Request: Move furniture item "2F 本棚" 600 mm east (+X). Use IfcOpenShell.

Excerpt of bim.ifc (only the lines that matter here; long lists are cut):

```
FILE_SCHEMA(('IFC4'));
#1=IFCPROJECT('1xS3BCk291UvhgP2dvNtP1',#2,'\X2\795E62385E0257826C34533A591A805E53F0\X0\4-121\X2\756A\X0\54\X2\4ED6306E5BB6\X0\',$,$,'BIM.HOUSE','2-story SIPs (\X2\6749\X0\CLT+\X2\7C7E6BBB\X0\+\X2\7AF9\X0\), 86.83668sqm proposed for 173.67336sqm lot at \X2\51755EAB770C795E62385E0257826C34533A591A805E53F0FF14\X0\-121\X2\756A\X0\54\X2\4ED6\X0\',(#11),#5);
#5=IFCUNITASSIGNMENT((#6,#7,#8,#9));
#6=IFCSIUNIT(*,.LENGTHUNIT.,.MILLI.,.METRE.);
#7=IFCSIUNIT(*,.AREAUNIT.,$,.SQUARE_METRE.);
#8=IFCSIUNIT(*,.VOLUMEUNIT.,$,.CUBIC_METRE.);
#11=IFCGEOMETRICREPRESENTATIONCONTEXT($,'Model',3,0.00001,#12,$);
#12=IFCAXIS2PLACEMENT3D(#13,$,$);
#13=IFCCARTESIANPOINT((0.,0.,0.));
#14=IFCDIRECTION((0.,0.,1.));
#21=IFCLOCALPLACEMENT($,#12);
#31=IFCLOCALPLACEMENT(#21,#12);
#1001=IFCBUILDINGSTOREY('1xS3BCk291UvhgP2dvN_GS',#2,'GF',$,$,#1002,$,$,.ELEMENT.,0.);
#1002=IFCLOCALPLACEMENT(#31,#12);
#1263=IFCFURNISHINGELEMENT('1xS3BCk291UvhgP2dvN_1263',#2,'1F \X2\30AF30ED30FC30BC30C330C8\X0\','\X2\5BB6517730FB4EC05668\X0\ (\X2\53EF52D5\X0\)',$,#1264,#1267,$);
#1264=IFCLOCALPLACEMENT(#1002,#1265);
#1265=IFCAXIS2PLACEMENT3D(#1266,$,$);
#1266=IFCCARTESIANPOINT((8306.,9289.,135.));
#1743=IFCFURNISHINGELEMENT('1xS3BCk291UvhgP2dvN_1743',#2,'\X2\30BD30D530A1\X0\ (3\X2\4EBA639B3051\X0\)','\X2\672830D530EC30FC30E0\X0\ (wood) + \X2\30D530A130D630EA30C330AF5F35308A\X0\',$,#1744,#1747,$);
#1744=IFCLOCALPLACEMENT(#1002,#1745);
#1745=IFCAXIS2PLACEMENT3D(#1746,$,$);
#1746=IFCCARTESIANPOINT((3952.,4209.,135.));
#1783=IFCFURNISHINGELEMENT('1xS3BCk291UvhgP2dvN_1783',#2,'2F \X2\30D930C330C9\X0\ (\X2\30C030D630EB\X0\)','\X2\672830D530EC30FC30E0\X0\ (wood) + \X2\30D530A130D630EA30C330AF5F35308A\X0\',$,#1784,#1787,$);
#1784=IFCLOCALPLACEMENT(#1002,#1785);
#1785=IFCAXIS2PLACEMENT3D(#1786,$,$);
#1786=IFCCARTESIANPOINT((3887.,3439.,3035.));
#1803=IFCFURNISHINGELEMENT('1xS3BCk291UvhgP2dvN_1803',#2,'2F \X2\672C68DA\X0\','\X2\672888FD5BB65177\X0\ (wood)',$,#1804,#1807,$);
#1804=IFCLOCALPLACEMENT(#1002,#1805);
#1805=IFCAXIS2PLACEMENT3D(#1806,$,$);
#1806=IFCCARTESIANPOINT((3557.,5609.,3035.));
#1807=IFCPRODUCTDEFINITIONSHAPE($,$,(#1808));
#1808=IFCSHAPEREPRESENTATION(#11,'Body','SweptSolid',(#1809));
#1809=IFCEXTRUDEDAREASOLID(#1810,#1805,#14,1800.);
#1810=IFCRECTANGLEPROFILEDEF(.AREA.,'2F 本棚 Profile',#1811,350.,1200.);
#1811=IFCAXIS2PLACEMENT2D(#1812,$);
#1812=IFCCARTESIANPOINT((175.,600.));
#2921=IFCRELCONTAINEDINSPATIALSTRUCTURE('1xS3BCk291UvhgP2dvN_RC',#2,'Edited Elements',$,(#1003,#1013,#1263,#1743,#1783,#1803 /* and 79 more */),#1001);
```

```python
import ifcopenshell
import ifcopenshell.api.geometry
import ifcopenshell.util.placement

model = ifcopenshell.open("bim.ifc")

item = model.by_id(1803)
matrix = ifcopenshell.util.placement.get_local_placement(item.ObjectPlacement)
matrix[0, 3] += 600.0
ifcopenshell.api.geometry.edit_object_placement(model, product=item, matrix=matrix, is_si=False)

print(ifcopenshell.util.placement.get_local_placement(item.ObjectPlacement).round(3) + 0.0)

model.write("bim_edited.ifc")
```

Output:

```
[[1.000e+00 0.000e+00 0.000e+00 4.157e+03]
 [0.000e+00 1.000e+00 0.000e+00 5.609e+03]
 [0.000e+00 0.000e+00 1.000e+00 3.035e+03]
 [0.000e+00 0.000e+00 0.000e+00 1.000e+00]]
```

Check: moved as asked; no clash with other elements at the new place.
